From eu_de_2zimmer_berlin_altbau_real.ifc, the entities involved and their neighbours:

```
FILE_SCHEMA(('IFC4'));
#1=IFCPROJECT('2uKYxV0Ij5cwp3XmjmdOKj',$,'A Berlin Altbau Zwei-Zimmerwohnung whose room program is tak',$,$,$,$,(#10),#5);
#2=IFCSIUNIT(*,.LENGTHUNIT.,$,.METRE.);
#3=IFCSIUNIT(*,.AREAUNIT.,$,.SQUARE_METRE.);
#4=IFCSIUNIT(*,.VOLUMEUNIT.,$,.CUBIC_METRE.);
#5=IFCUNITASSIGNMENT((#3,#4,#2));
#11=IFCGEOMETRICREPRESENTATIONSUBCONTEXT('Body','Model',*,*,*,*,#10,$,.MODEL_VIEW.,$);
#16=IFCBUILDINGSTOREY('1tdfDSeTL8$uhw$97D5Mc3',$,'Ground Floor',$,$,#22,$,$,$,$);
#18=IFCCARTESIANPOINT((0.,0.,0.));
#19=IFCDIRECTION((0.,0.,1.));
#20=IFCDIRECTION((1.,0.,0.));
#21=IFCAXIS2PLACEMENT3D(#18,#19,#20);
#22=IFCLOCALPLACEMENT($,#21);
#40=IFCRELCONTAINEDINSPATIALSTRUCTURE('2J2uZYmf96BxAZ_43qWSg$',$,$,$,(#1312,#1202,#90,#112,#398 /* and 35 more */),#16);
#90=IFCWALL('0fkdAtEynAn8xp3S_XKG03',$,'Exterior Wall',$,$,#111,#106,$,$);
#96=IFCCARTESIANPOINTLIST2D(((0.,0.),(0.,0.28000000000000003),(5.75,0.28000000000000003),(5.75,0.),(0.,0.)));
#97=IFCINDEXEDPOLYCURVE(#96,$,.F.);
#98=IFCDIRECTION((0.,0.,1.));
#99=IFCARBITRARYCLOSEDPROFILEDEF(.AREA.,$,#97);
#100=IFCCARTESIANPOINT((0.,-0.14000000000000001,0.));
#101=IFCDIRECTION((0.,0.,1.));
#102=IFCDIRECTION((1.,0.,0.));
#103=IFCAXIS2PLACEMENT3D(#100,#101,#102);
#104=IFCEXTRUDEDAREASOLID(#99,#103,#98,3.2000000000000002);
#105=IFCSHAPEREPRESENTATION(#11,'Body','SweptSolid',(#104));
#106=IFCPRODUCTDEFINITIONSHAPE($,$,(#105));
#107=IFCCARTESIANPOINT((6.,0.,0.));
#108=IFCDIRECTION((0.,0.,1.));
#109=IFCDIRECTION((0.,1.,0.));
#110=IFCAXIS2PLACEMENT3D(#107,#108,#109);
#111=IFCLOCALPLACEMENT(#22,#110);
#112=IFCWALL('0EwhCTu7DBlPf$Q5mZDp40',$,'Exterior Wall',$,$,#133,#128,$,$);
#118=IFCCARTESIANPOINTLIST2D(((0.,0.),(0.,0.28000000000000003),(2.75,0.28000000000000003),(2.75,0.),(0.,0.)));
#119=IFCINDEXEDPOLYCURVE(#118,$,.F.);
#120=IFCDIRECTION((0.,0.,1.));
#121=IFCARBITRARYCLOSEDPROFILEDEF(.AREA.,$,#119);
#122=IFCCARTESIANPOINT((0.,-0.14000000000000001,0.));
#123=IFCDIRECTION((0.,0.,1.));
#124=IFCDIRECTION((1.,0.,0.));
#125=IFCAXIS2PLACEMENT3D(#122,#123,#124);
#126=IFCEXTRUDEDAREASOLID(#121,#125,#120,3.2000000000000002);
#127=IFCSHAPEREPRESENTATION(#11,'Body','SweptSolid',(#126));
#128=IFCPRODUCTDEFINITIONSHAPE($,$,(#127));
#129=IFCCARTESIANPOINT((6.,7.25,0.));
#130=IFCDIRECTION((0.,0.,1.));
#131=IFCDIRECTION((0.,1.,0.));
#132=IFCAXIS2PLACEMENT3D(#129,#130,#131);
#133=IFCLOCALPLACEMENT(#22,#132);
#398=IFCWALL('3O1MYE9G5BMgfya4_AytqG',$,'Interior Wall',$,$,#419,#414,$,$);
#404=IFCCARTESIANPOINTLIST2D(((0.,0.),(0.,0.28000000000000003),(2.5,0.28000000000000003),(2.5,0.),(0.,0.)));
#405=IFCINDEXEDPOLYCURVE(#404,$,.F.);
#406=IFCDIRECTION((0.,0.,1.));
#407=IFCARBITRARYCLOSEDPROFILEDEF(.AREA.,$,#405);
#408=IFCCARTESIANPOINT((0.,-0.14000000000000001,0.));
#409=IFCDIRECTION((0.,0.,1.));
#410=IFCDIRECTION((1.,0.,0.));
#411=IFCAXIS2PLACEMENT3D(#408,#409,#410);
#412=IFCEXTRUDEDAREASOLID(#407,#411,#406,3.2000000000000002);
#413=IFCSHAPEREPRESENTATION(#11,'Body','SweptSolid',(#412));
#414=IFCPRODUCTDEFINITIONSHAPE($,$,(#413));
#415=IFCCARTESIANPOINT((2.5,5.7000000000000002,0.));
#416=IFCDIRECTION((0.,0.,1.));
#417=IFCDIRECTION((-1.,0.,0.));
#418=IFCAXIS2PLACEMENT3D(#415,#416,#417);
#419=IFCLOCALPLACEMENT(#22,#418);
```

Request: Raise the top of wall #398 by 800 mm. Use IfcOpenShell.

```python
import ifcopenshell
import ifcopenshell.geom
import ifcopenshell.util.representation
import ifcopenshell.util.shape

model = ifcopenshell.open("eu_de_2zimmer_berlin_altbau_real.ifc")
settings = ifcopenshell.geom.settings()


def volume(element):
    """Net volume in cubic metres, openings subtracted."""
    shape = ifcopenshell.geom.create_shape(settings, element)
    return ifcopenshell.util.shape.get_volume(shape.geometry)


wall = model.by_id(398)
before = volume(wall)

body = ifcopenshell.util.representation.get_representation(wall, "Model", "Body")
solid = body.Items[0]
old_height = solid.Depth
solid.Depth += 0.8
after = volume(wall)

print(f"height {old_height:g} -> {solid.Depth:g}, volume {before:.3f} -> {after:.3f} m3")

model.write("eu_de_2zimmer_berlin_altbau_real_edited.ifc")
```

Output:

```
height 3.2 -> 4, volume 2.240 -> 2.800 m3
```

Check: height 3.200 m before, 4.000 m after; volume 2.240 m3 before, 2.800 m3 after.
